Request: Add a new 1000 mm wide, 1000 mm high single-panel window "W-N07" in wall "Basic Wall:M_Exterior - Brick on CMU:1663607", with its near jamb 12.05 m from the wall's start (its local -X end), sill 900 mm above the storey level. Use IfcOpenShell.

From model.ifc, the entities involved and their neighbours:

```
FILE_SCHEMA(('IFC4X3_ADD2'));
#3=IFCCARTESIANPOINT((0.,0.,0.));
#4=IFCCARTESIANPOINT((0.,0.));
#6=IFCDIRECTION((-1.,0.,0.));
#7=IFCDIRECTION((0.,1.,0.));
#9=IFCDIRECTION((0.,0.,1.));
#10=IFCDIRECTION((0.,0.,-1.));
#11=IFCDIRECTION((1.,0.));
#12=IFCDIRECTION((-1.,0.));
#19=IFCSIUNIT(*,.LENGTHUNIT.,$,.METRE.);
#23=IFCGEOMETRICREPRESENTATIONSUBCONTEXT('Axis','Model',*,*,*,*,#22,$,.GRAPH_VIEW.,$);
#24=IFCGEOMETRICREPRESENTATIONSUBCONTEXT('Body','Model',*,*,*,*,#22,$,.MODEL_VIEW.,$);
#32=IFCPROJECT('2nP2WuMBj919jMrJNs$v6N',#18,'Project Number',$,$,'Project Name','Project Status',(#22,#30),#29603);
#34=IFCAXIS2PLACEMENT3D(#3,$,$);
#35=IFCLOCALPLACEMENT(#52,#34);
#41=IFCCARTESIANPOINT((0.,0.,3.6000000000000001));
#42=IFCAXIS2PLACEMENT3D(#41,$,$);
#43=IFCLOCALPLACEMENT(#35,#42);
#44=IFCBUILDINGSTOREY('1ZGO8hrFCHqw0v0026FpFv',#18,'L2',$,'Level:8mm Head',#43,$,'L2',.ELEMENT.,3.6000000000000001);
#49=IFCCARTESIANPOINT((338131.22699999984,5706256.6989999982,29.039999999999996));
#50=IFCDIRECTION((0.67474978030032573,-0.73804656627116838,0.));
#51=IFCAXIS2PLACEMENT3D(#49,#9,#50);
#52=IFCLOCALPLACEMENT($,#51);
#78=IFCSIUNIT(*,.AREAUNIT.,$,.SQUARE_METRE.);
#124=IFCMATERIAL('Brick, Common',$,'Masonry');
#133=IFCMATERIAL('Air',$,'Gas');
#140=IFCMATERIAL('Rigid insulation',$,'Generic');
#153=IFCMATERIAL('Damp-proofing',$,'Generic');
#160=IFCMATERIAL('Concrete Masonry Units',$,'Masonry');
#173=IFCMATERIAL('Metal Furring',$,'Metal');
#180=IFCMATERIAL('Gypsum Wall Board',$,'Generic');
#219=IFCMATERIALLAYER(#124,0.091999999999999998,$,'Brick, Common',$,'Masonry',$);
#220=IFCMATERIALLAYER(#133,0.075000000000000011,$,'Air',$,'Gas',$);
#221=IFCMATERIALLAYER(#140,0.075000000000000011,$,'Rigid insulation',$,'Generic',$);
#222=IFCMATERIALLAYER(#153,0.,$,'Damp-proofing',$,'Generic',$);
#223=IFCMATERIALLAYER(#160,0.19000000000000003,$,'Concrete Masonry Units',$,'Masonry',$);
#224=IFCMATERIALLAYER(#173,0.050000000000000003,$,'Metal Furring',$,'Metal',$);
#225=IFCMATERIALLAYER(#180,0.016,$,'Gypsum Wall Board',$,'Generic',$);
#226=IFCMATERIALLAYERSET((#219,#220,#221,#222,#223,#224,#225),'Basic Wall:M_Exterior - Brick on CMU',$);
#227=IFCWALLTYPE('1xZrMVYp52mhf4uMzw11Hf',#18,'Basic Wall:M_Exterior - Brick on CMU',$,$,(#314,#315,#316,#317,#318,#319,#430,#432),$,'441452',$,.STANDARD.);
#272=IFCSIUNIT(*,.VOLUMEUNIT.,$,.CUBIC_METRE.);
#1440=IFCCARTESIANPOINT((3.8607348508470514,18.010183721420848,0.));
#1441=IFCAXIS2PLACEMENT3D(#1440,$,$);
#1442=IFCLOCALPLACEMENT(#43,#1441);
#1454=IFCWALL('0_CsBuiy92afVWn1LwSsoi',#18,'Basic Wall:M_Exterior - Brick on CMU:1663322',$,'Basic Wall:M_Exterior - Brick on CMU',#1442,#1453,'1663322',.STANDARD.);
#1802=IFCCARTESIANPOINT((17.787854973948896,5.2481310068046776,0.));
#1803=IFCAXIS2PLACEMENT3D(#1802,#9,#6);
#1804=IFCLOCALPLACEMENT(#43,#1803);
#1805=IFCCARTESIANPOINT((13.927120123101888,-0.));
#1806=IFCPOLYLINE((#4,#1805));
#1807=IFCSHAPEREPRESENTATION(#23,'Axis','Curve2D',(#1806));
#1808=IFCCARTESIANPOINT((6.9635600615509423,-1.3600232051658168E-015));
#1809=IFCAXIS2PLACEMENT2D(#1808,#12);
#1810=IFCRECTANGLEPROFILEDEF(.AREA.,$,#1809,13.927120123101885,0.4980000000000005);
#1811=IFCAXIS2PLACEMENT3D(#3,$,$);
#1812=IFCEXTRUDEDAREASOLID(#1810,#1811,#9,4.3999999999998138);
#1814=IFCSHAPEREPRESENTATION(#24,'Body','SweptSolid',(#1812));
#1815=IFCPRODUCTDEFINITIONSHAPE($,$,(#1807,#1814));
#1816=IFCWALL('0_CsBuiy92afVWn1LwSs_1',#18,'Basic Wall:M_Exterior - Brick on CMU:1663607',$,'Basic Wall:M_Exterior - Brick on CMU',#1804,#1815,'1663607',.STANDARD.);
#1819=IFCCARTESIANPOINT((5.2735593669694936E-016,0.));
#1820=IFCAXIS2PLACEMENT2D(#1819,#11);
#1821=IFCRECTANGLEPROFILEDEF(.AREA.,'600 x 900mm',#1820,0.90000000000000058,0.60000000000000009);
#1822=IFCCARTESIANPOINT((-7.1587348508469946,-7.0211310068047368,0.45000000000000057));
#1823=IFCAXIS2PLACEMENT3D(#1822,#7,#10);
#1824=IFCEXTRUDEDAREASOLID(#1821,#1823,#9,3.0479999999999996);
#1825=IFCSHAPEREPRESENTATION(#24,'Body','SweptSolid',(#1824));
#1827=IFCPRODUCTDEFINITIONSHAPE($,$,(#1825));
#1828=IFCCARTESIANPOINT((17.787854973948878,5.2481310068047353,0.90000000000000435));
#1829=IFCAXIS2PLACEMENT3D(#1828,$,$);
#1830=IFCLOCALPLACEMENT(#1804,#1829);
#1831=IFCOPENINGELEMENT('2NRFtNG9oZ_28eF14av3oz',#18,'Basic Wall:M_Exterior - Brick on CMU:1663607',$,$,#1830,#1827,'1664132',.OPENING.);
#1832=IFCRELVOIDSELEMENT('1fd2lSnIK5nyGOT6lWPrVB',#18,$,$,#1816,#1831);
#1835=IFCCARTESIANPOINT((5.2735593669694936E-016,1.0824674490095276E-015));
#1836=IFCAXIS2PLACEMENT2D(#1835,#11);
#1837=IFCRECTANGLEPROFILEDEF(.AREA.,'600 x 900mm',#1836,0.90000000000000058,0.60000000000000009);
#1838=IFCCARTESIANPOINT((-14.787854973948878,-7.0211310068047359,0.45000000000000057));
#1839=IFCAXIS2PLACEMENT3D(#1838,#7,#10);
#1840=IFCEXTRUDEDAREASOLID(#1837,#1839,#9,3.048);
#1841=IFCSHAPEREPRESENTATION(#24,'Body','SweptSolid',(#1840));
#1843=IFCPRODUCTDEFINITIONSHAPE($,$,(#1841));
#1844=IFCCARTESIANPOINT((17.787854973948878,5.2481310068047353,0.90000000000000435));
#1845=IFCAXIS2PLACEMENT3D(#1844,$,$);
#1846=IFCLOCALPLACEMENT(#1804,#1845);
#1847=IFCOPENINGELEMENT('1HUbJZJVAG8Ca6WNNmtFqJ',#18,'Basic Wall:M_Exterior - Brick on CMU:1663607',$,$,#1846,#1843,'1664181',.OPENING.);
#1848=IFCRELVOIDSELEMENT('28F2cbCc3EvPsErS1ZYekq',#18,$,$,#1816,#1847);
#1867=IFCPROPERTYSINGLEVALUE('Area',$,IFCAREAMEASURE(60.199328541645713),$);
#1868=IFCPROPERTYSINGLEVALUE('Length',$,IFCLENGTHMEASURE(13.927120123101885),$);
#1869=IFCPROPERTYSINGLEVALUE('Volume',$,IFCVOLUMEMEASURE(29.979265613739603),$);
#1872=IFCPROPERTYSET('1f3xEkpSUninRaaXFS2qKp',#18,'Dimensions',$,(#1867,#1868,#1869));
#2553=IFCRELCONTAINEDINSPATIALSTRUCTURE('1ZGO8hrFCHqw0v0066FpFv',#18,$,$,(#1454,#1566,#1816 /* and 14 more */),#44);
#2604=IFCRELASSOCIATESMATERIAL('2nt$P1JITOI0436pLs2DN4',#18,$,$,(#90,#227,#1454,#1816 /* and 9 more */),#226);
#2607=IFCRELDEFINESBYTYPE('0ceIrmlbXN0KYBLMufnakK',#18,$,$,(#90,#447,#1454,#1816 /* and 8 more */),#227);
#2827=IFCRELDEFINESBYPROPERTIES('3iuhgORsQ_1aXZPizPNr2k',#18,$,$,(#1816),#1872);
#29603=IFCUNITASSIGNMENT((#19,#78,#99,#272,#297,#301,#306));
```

```python
import numpy as np
import ifcopenshell
import ifcopenshell.api.feature
import ifcopenshell.api.geometry
import ifcopenshell.api.pset
import ifcopenshell.api.root
import ifcopenshell.api.spatial
import ifcopenshell.geom
import ifcopenshell.util.element
import ifcopenshell.util.placement
import ifcopenshell.util.representation
import ifcopenshell.util.shape
import ifcopenshell.util.unit

model = ifcopenshell.open("model.ifc")
unit_scale = ifcopenshell.util.unit.calculate_unit_scale(model)
area_scale = ifcopenshell.util.unit.calculate_unit_scale(model, "AREAUNIT")
volume_scale = ifcopenshell.util.unit.calculate_unit_scale(model, "VOLUMEUNIT")
settings = ifcopenshell.geom.settings()


def volume(element):
    """Net volume in cubic metres, openings subtracted."""
    shape = ifcopenshell.geom.create_shape(settings, element)
    return ifcopenshell.util.shape.get_volume(shape.geometry)


wall = model.by_guid("0_CsBuiy92afVWn1LwSs_1")
storey = ifcopenshell.util.element.get_container(wall, ifc_class="IfcBuildingStorey")
context = ifcopenshell.util.representation.get_context(model, "Model", "Body", "MODEL_VIEW")
before = volume(wall)

width, height, from_end, sill = 1, 1, 12.05, 0.9  # metres

# The wall runs along its own X axis, and the end named is its -X end.
wall_shape = ifcopenshell.geom.create_shape(settings, wall)
x, y, z = ifcopenshell.util.shape.get_vertices(wall_shape.geometry).T
start = x.min() + from_end
face, thickness = float(y.min()), float(y.max() - y.min())
wall_matrix = ifcopenshell.util.placement.get_local_placement(wall.ObjectPlacement)
level = ifcopenshell.util.placement.get_local_placement(storey.ObjectPlacement)[2, 3]


def in_wall(x, y):
    """Placement at x, y metres in the wall's axes, at sill height."""
    matrix = wall_matrix.copy()
    matrix[:, 3] = wall_matrix @ np.array([x / unit_scale, y / unit_scale, 0.0, 1.0])
    matrix[2, 3] = level + sill / unit_scale
    return matrix


# Opening: a box that overshoots both wall faces by 50 mm.
opening = ifcopenshell.api.root.create_entity(model, ifc_class="IfcOpeningElement", predefined_type="OPENING")
box = ifcopenshell.api.geometry.add_wall_representation(
    model, context=context, length=width, height=height, thickness=thickness + 0.1
)
ifcopenshell.api.geometry.assign_representation(model, product=opening, representation=box)
ifcopenshell.api.geometry.edit_object_placement(model, product=opening, matrix=in_wall(start, face - 0.05), is_si=False)
ifcopenshell.api.feature.add_feature(model, feature=opening, element=wall)

window = ifcopenshell.api.root.create_entity(model, ifc_class="IfcWindow", name="W-N07", predefined_type="WINDOW")
window.OverallWidth, window.OverallHeight = width / unit_scale, height / unit_scale
window.PartitioningType = "SINGLE_PANEL"
body = ifcopenshell.api.geometry.add_window_representation(
    model,
    context=context,
    overall_width=window.OverallWidth,
    overall_height=window.OverallHeight,
    partition_type="SINGLE_PANEL",
)
ifcopenshell.api.geometry.assign_representation(model, product=window, representation=body)
ifcopenshell.api.spatial.assign_container(model, products=[window], relating_structure=storey)
ifcopenshell.api.feature.add_filling(model, opening=opening, element=window)

# Centre the window in the wall's thickness.
ifcopenshell.api.geometry.edit_object_placement(model, product=window, matrix=in_wall(start, face), is_si=False)
window_shape = ifcopenshell.geom.create_shape(settings, window)
depth = ifcopenshell.util.shape.get_vertices(window_shape.geometry)[:, 1]
offset = face + thickness / 2 - (depth.min() + depth.max()) / 2
ifcopenshell.api.geometry.edit_object_placement(model, product=window, matrix=in_wall(start, offset), is_si=False)

after = volume(wall)

# Update the wall's stored quantities.
pset = model.by_id(ifcopenshell.util.element.get_pset(wall, "Dimensions", should_inherit=False)["id"])
ifcopenshell.api.pset.edit_pset(model, pset=pset, properties={
    "Area": model.create_entity("IfcAreaMeasure", after / thickness / area_scale),
    "Volume": model.create_entity("IfcVolumeMeasure", after / volume_scale),
})

print(f"wall volume {before:.3f} -> {after:.3f} m3")

model.write("model-out.ifc")
```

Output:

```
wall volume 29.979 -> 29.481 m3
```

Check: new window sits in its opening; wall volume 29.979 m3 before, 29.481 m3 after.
